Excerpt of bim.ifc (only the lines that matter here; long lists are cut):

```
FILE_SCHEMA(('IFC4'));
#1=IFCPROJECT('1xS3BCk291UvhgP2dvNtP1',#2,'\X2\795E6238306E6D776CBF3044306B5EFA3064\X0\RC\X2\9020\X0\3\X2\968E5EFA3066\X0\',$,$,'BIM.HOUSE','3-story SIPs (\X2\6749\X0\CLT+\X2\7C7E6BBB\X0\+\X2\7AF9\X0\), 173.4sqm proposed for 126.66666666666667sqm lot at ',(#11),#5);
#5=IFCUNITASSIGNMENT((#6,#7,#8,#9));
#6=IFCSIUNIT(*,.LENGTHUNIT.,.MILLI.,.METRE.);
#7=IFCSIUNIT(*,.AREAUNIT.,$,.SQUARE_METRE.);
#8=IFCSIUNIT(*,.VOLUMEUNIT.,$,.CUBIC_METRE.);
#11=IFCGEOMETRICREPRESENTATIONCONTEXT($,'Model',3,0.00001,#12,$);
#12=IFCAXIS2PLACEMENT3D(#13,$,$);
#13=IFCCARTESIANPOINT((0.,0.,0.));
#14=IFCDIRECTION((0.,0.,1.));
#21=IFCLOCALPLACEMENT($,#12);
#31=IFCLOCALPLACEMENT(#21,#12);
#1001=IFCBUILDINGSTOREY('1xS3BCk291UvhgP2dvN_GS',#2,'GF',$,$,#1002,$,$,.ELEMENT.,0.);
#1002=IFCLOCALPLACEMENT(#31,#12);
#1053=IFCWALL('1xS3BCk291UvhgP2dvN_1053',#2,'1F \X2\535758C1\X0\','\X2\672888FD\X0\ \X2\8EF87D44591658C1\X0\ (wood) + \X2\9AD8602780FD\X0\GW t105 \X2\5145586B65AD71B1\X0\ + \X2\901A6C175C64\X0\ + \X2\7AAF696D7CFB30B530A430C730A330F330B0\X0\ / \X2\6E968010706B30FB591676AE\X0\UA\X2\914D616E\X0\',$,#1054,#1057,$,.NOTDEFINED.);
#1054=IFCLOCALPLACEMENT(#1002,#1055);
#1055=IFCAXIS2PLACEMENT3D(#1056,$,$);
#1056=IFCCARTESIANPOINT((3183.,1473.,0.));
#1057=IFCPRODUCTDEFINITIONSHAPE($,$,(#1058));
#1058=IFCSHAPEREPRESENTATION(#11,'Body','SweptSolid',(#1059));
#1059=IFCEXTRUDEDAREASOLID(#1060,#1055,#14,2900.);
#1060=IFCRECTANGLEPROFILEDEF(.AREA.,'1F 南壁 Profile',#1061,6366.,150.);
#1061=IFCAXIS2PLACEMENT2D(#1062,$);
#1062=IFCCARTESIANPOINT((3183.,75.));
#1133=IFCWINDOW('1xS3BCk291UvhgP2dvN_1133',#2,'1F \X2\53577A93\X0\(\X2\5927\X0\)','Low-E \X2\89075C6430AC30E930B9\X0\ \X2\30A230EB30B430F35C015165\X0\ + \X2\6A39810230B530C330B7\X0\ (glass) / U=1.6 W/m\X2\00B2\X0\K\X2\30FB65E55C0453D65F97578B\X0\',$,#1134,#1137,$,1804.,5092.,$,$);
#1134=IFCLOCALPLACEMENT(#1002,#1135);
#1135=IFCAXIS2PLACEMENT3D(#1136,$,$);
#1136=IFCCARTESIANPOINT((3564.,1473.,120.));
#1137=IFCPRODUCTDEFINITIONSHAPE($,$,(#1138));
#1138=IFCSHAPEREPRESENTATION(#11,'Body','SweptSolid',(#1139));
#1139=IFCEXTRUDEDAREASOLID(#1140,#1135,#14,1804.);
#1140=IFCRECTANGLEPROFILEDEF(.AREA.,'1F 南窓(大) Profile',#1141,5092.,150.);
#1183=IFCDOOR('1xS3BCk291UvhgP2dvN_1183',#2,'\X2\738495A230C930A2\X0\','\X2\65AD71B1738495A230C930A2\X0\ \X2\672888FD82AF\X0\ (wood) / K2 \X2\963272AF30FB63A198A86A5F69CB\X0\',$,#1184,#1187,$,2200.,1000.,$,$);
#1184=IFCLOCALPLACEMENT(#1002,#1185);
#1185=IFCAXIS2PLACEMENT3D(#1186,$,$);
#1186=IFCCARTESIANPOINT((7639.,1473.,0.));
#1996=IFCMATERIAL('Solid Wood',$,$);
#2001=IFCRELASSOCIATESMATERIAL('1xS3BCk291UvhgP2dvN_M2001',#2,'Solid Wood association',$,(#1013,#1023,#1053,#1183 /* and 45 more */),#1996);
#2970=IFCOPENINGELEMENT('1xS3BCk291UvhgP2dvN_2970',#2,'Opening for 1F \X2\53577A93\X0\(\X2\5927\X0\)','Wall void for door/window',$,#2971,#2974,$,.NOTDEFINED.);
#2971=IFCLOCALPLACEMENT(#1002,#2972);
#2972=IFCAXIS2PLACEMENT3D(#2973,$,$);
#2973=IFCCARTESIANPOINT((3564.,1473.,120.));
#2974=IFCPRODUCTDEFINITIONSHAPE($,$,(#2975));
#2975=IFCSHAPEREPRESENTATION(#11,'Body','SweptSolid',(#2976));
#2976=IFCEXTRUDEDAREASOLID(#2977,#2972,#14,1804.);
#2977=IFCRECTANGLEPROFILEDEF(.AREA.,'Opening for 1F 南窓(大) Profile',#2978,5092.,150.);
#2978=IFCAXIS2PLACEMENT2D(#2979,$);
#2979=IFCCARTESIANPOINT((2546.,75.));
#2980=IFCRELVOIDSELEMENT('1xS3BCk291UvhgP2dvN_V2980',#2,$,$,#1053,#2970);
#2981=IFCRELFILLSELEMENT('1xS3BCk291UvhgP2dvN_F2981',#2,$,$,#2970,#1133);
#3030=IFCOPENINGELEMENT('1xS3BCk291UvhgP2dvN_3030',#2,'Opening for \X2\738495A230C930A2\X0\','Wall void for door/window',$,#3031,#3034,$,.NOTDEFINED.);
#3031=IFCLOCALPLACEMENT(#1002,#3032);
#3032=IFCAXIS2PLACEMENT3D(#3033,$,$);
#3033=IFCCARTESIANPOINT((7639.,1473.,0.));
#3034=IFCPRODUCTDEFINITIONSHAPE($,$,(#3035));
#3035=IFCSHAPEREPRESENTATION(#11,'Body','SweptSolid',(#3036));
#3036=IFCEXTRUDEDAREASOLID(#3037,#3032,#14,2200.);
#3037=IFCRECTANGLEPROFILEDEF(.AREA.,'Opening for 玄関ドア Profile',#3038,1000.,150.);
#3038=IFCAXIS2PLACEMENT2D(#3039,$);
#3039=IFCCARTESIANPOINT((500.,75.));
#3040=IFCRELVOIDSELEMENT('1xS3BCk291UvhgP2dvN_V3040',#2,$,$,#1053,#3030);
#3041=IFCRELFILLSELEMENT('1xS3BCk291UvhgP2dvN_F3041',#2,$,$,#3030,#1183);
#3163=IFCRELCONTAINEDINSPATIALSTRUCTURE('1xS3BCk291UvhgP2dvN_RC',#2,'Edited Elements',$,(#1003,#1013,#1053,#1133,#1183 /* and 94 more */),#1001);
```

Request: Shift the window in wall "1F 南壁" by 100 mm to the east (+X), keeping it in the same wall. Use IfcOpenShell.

```python
import ifcopenshell
import ifcopenshell.api.geometry
import ifcopenshell.util.placement

model = ifcopenshell.open("bim.ifc")

window = model.by_id(1133)
opening = window.FillsVoids[0].RelatingOpeningElement
wall = opening.VoidsElements[0].RelatingBuildingElement

wall_matrix = ifcopenshell.util.placement.get_local_placement(wall.ObjectPlacement)
shift = wall_matrix[:3, 0] * 100.0
before = ifcopenshell.util.placement.get_local_placement(window.ObjectPlacement)[:3, 3].copy()

# The window is not placed relative to its opening, so move both.
for product in (opening, window):
    matrix = ifcopenshell.util.placement.get_local_placement(product.ObjectPlacement)
    matrix[:3, 3] += shift
    ifcopenshell.api.geometry.edit_object_placement(model, product=product, matrix=matrix, is_si=False)

after = ifcopenshell.util.placement.get_local_placement(window.ObjectPlacement)[:3, 3]
print("window moved by", (after - before).round(3) + 0.0)

model.write("bim_edited.ifc")
```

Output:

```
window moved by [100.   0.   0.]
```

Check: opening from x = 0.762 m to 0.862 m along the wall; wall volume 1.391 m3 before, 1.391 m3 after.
